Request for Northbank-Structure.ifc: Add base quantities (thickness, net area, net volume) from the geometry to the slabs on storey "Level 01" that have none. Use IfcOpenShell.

First a look at what the model holds.

```python
import ifcopenshell
import ifcopenshell.util.element
import ifcopenshell.util.unit

model = ifcopenshell.open("Northbank-Structure.ifc")
print(model.schema)
for unit_type in ("LENGTHUNIT", "AREAUNIT", "VOLUMEUNIT"):
    print(unit_type, ifcopenshell.util.unit.calculate_unit_scale(model, unit_type))
storey = next(s for s in model.by_type("IfcBuildingStorey") if s.Name == "Level 01")
slabs = [e for e in ifcopenshell.util.element.get_decomposition(storey) if e.is_a("IfcSlab")]
for e in sorted(slabs, key=lambda e: e.id()):
    print(e.id(), e.is_a(), e.Name, list(ifcopenshell.util.element.get_psets(e, qtos_only=True)), sep=" | ")
```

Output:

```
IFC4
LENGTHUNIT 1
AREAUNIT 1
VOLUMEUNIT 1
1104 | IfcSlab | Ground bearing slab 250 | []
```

```python
import ifcopenshell
import ifcopenshell.api.pset
import ifcopenshell.geom
import ifcopenshell.util.element
import ifcopenshell.util.shape
import ifcopenshell.util.unit

model = ifcopenshell.open("Northbank-Structure.ifc")
unit_scale = ifcopenshell.util.unit.calculate_unit_scale(model)
area_scale = ifcopenshell.util.unit.calculate_unit_scale(model, "AREAUNIT")
volume_scale = ifcopenshell.util.unit.calculate_unit_scale(model, "VOLUMEUNIT")
settings = ifcopenshell.geom.settings()

storey = next(s for s in model.by_type("IfcBuildingStorey") if s.Name == "Level 01")
slabs = [e for e in ifcopenshell.util.element.get_decomposition(storey) if e.is_a("IfcSlab")]

for e in sorted(slabs, key=lambda e: e.id()):
    if ifcopenshell.util.element.get_psets(e, qtos_only=True, should_inherit=False):
        continue
    # Geometry comes back in metres, in the element's own axes.
    shape = ifcopenshell.geom.create_shape(settings, e)
    values = {
        "Width": ifcopenshell.util.shape.get_z(shape.geometry) / unit_scale,
        "NetArea": ifcopenshell.util.shape.get_footprint_area(shape.geometry) / area_scale,
        "NetVolume": ifcopenshell.util.shape.get_volume(shape.geometry) / volume_scale,
    }
    qto = ifcopenshell.api.pset.add_qto(model, product=e, name="Qto_SlabBaseQuantities")
    ifcopenshell.api.pset.edit_qto(model, qto=qto, properties=values)
    print(e.id(), {k: round(v, 3) for k, v in values.items()})

model.write("Northbank-Structure_updated.ifc")
```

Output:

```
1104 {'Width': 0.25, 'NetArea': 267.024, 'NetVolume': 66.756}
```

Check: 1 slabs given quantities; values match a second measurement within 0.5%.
